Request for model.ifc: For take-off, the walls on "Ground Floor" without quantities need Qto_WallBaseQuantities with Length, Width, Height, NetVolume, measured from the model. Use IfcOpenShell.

First a look at what the model holds.

```python
import ifcopenshell
import ifcopenshell.util.element
import ifcopenshell.util.unit

model = ifcopenshell.open("model.ifc")
print(model.schema)
for unit_type in ("LENGTHUNIT", "AREAUNIT", "VOLUMEUNIT"):
    print(unit_type, ifcopenshell.util.unit.calculate_unit_scale(model, unit_type))
storey = next(s for s in model.by_type("IfcBuildingStorey") if s.Name == "Ground Floor")
walls = [e for e in ifcopenshell.util.element.get_decomposition(storey) if e.is_a("IfcWall")]
for e in sorted(walls, key=lambda e: e.id()):
    print(e.id(), e.is_a(), e.Name, list(ifcopenshell.util.element.get_psets(e, qtos_only=True)), sep=" | ")
```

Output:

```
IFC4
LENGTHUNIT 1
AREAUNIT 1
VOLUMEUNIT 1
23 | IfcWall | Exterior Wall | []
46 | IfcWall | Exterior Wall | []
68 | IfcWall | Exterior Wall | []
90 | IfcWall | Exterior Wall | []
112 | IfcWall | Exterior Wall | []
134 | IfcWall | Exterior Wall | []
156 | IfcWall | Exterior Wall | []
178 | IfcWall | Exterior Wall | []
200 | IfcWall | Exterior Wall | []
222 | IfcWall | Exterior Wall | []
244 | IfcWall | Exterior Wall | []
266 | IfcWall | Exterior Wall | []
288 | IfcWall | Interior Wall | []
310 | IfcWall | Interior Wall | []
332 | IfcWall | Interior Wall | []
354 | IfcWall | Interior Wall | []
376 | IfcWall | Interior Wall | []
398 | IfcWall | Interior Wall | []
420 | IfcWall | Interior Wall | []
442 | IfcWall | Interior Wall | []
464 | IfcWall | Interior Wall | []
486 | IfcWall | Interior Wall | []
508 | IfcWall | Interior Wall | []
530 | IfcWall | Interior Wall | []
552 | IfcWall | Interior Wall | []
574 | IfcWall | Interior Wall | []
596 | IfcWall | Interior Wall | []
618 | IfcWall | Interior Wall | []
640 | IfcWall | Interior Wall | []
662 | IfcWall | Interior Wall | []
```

```python
import ifcopenshell
import ifcopenshell.api.pset
import ifcopenshell.geom
import ifcopenshell.util.element
import ifcopenshell.util.shape
import ifcopenshell.util.unit

model = ifcopenshell.open("model.ifc")
unit_scale = ifcopenshell.util.unit.calculate_unit_scale(model)
volume_scale = ifcopenshell.util.unit.calculate_unit_scale(model, "VOLUMEUNIT")
settings = ifcopenshell.geom.settings()

storey = next(s for s in model.by_type("IfcBuildingStorey") if s.Name == "Ground Floor")
walls = [e for e in ifcopenshell.util.element.get_decomposition(storey) if e.is_a("IfcWall")]

for e in sorted(walls, key=lambda e: e.id()):
    if ifcopenshell.util.element.get_psets(e, qtos_only=True, should_inherit=False):
        continue
    # Geometry comes back in metres, in the element's own axes.
    shape = ifcopenshell.geom.create_shape(settings, e)
    values = {
        "Length": ifcopenshell.util.shape.get_x(shape.geometry) / unit_scale,
        "Width": ifcopenshell.util.shape.get_y(shape.geometry) / unit_scale,
        "Height": ifcopenshell.util.shape.get_z(shape.geometry) / unit_scale,
        "NetVolume": ifcopenshell.util.shape.get_volume(shape.geometry) / volume_scale,
    }
    qto = ifcopenshell.api.pset.add_qto(model, product=e, name="Qto_WallBaseQuantities")
    ifcopenshell.api.pset.edit_qto(model, qto=qto, properties=values)
    print(e.id(), {k: round(v, 3) for k, v in values.items()})

model.write("model_edited.ifc")
```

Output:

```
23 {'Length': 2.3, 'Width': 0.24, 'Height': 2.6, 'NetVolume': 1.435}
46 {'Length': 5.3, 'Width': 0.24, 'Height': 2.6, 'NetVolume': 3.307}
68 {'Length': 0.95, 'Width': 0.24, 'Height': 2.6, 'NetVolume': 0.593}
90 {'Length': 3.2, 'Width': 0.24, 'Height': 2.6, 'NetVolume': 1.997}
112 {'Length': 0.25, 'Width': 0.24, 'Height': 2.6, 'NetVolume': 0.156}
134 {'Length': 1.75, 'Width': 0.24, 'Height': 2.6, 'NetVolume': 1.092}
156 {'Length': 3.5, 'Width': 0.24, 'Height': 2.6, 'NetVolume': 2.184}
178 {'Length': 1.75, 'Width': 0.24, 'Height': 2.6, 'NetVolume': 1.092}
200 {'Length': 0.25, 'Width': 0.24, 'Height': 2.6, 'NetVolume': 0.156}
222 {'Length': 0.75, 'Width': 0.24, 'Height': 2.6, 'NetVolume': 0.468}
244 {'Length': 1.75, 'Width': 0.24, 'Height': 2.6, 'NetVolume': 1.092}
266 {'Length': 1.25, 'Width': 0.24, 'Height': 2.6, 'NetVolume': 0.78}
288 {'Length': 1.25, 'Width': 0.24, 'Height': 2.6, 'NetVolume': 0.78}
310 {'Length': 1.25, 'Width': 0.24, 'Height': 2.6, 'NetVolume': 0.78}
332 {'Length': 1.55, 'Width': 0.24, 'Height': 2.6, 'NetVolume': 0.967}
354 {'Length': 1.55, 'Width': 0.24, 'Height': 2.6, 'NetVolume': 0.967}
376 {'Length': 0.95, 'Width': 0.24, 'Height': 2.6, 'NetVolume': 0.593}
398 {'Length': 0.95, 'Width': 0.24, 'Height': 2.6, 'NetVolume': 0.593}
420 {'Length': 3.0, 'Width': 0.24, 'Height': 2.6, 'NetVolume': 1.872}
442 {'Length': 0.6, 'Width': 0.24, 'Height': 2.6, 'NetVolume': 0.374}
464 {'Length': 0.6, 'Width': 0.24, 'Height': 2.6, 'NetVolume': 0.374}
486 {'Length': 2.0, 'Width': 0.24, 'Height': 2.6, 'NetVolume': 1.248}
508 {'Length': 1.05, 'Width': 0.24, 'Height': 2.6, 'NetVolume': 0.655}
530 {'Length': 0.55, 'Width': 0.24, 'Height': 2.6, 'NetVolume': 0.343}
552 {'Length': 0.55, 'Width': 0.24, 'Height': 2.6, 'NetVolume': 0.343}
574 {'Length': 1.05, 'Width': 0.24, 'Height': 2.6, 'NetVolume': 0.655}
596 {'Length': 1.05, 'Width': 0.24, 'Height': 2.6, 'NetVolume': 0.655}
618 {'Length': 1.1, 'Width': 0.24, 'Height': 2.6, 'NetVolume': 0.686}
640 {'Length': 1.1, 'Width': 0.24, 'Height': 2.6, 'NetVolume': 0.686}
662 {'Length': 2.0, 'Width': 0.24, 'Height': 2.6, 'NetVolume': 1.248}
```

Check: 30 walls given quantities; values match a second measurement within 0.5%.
